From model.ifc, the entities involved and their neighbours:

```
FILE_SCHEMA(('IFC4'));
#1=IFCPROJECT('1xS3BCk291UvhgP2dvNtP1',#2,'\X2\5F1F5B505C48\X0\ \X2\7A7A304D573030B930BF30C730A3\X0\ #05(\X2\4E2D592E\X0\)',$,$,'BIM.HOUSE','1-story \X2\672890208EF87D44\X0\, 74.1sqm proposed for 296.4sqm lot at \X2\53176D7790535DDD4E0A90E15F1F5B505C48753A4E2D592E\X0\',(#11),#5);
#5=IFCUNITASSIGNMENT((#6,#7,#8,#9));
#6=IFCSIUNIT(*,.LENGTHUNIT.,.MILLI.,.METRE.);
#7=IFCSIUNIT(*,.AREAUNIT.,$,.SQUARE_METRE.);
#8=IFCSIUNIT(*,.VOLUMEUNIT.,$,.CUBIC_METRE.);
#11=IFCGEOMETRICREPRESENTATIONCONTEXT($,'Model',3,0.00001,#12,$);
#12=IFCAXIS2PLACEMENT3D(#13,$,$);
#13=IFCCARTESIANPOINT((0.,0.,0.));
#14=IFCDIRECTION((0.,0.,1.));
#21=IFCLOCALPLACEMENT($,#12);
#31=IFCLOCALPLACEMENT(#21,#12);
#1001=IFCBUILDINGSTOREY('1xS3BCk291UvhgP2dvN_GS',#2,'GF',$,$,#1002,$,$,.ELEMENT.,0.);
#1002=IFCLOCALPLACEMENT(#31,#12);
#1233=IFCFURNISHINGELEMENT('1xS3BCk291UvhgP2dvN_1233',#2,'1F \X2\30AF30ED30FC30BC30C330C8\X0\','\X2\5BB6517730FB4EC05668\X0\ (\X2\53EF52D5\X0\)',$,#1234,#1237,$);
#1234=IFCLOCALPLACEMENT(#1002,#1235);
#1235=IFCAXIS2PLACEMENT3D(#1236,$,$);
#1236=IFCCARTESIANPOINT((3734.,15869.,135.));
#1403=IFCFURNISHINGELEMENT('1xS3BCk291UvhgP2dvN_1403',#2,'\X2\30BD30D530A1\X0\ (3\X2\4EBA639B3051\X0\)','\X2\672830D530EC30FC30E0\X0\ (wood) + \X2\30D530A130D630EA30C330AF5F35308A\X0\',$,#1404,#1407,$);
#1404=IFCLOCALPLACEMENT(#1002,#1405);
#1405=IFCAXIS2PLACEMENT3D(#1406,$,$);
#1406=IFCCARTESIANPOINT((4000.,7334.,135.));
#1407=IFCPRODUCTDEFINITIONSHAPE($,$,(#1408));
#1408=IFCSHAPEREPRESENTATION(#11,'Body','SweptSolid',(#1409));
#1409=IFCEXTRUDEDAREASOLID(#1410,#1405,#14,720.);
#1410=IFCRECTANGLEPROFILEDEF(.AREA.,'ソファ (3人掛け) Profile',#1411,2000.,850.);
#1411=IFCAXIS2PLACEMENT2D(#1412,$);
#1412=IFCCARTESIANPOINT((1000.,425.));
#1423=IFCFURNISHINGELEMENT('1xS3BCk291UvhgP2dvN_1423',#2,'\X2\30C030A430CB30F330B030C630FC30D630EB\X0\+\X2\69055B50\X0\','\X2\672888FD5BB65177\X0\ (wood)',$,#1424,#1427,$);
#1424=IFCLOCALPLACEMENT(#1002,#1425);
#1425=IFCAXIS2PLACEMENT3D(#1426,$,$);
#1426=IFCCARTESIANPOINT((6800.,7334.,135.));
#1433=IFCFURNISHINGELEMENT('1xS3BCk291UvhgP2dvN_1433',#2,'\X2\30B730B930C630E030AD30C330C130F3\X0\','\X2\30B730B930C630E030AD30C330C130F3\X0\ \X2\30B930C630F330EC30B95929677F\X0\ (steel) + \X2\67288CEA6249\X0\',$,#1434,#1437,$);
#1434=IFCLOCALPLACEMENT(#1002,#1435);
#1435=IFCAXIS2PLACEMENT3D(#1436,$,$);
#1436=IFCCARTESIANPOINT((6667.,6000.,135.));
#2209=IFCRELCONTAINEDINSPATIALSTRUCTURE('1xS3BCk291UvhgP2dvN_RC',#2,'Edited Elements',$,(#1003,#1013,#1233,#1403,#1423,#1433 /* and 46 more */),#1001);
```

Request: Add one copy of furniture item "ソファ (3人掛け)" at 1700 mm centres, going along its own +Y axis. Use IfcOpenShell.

```python
import ifcopenshell
import ifcopenshell.api.geometry
import ifcopenshell.api.root
import ifcopenshell.util.element
import ifcopenshell.util.placement
import ifcopenshell.util.unit

model = ifcopenshell.open("model.ifc")
unit_scale = ifcopenshell.util.unit.calculate_unit_scale(model)


def reuse_history(source, copy):
    """copy_class also copies each property set's owner history, people and application; keep the originals."""
    for rel in copy.IsDefinedBy:
        if rel.is_a("IfcRelDefinesByProperties") and (history := rel.RelatingPropertyDefinition.OwnerHistory):
            rel.RelatingPropertyDefinition.OwnerHistory = source.OwnerHistory
            ifcopenshell.util.element.remove_deep2(model, history)


source = model.by_guid("1xS3BCk291UvhgP2dvN_1403")
base = ifcopenshell.util.placement.get_local_placement(source.ObjectPlacement)
step = base[:3, 1] * 1.7 / unit_scale

for i in range(1, 2):
    copy = ifcopenshell.api.root.copy_class(model, product=source)
    copy.Representation = ifcopenshell.util.element.copy_deep(
        model, source.Representation, exclude=["IfcGeometricRepresentationContext", "IfcRepresentationMap"]
    )
    reuse_history(source, copy)
    matrix = base.copy()
    matrix[:3, 3] += i * step
    print("added at", matrix[:3, 3].round(3) + 0.0)
    ifcopenshell.api.geometry.edit_object_placement(model, product=copy, matrix=matrix, is_si=False)

model.write("model_v2.ifc")
```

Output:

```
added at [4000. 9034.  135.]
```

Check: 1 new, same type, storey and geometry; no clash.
